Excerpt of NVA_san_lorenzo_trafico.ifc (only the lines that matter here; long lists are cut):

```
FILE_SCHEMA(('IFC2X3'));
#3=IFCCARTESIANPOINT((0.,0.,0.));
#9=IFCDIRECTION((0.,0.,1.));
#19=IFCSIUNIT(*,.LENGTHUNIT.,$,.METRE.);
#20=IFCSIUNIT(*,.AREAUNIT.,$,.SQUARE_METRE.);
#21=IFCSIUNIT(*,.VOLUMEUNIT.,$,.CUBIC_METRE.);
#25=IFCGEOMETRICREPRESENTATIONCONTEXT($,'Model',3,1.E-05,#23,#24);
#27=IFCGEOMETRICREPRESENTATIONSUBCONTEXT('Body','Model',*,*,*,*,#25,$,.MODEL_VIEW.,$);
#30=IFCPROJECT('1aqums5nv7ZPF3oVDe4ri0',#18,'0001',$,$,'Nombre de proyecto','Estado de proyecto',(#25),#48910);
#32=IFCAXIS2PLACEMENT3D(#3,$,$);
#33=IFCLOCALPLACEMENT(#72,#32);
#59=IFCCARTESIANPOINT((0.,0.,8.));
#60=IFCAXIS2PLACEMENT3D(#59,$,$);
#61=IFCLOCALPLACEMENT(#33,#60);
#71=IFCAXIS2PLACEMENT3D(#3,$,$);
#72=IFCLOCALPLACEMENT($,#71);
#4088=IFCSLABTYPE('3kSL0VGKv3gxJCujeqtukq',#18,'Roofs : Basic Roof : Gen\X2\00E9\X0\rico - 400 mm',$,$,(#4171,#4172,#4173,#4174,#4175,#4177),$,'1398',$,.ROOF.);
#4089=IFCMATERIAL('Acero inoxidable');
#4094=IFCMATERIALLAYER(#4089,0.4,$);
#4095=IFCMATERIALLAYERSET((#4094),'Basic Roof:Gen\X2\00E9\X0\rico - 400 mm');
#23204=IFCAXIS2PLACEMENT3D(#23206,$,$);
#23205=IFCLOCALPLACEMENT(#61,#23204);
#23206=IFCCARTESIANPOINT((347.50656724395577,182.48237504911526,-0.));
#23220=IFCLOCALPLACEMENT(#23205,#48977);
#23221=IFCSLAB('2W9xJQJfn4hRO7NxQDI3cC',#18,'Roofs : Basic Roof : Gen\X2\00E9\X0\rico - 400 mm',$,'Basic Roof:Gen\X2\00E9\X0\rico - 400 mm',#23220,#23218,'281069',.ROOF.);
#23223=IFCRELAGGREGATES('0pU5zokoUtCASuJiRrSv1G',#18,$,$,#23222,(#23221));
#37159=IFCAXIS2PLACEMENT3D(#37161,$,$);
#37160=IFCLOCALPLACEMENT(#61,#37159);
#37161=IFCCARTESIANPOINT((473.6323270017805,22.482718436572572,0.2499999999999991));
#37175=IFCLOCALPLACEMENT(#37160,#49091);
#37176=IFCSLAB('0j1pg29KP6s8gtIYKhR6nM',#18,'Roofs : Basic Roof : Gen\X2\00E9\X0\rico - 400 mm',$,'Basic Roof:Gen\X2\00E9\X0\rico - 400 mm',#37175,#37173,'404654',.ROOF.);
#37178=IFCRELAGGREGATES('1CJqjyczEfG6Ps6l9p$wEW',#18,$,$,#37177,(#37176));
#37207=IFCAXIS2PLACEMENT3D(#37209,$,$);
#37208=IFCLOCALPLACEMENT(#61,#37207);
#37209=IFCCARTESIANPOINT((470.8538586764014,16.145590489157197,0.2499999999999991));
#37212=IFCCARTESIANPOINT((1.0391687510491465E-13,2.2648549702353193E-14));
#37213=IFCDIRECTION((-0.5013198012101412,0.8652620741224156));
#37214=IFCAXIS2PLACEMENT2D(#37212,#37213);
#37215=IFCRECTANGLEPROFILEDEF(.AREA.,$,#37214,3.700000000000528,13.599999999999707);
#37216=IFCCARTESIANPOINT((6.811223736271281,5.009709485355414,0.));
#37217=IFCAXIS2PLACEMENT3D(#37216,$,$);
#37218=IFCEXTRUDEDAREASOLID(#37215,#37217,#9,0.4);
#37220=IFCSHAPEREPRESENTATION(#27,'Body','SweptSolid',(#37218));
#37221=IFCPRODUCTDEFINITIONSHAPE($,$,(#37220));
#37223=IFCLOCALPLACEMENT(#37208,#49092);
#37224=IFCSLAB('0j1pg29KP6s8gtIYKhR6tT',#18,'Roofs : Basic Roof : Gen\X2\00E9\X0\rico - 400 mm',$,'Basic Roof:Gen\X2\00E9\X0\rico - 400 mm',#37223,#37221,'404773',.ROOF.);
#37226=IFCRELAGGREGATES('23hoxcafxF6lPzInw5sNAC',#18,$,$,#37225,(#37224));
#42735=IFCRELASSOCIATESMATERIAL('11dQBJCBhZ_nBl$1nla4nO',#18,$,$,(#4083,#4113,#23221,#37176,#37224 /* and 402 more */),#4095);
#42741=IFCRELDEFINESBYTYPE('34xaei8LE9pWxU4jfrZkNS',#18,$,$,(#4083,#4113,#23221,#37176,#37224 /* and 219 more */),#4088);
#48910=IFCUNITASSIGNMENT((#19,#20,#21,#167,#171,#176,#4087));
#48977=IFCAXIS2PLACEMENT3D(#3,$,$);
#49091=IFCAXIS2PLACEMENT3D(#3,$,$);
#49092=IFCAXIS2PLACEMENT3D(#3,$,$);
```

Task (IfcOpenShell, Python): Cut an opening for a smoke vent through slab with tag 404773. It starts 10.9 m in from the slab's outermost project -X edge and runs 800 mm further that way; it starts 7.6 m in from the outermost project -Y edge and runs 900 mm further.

```python
import numpy as np
import ifcopenshell
import ifcopenshell.api.feature
import ifcopenshell.api.geometry
import ifcopenshell.api.root
import ifcopenshell.geom
import ifcopenshell.util.placement
import ifcopenshell.util.representation
import ifcopenshell.util.shape
import ifcopenshell.util.unit

model = ifcopenshell.open("NVA_san_lorenzo_trafico.ifc")
unit_scale = ifcopenshell.util.unit.calculate_unit_scale(model)
settings = ifcopenshell.geom.settings()


def volume(element):
    """Net volume in cubic metres, openings subtracted."""
    shape = ifcopenshell.geom.create_shape(settings, element)
    return ifcopenshell.util.shape.get_volume(shape.geometry)


slab = model.by_guid("0j1pg29KP6s8gtIYKhR6tT")
before = volume(slab)

# Extent in the slab's own axes, in metres. The edges named are its -X and -Y sides.
slab_shape = ifcopenshell.geom.create_shape(settings, slab)
vertices = ifcopenshell.util.shape.get_vertices(slab_shape.geometry)
x_min, y_min, bottom = vertices.min(axis=0)
top = vertices[:, 2].max()

opening = ifcopenshell.api.root.create_entity(model, ifc_class="IfcOpeningElement", name="Smoke vent opening")
context = ifcopenshell.util.representation.get_context(model, "Model", "Body", "MODEL_VIEW")
width, depth = 0.8, 0.9
outline = [(0.0, 0.0), (width, 0.0), (width, depth), (0.0, depth), (0.0, 0.0)]
# Overshoot both faces by 50 mm so the cut is clean.
shape = ifcopenshell.api.geometry.add_slab_representation(
    model, context=context, depth=top - bottom + 0.1, polyline=outline
)
ifcopenshell.api.geometry.assign_representation(model, product=opening, representation=shape)

matrix = ifcopenshell.util.placement.get_local_placement(slab.ObjectPlacement)
matrix[:, 3] = matrix @ np.append(np.array([x_min + 10.9, y_min + 7.6, bottom - 0.05]) / unit_scale, 1.0)
ifcopenshell.api.geometry.edit_object_placement(model, product=opening, matrix=matrix, is_si=False)
ifcopenshell.api.feature.add_feature(model, feature=opening, element=slab)

after = volume(slab)

print(f"slab volume {before:.3f} -> {after:.3f} m3")

model.write("NVA_san_lorenzo_trafico_updated.ifc")
```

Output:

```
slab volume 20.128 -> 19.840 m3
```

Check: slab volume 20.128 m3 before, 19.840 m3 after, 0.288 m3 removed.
